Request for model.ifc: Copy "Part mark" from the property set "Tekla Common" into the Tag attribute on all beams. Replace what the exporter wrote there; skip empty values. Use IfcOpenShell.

First a look at what the model holds.

```python
import ifcopenshell
import ifcopenshell.util.element

model = ifcopenshell.open("model.ifc")
print(model.schema)
beams = model.by_type("IfcBeam")
print(len(beams), "beams")
for e in beams[:8]:
    source = ifcopenshell.util.element.get_pset(e, "Tekla Common", "Part mark")
    target = e.Tag
    print(e.id(), repr(source), repr(target), sep=" | ")
```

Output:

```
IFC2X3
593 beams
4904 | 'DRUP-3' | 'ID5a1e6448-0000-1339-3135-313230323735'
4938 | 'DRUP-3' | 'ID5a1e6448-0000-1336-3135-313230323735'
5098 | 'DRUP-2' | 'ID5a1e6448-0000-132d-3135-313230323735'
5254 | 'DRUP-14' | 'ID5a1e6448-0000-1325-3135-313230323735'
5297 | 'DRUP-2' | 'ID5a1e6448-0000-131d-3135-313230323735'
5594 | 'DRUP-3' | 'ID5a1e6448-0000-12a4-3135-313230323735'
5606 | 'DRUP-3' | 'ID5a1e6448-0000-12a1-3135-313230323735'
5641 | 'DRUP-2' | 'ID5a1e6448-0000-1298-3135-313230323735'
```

```python
import ifcopenshell
import ifcopenshell.util.element

model = ifcopenshell.open("model.ifc")

count = 0
for e in model.by_type("IfcBeam"):
    value = ifcopenshell.util.element.get_pset(e, "Tekla Common", "Part mark")
    current = e.Tag
    if not value or not value.strip() or current == value:
        continue
    e.Tag = value
    count += 1

print(count, "beams updated")

model.write("model_rev.ifc")
```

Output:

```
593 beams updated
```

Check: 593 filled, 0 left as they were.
